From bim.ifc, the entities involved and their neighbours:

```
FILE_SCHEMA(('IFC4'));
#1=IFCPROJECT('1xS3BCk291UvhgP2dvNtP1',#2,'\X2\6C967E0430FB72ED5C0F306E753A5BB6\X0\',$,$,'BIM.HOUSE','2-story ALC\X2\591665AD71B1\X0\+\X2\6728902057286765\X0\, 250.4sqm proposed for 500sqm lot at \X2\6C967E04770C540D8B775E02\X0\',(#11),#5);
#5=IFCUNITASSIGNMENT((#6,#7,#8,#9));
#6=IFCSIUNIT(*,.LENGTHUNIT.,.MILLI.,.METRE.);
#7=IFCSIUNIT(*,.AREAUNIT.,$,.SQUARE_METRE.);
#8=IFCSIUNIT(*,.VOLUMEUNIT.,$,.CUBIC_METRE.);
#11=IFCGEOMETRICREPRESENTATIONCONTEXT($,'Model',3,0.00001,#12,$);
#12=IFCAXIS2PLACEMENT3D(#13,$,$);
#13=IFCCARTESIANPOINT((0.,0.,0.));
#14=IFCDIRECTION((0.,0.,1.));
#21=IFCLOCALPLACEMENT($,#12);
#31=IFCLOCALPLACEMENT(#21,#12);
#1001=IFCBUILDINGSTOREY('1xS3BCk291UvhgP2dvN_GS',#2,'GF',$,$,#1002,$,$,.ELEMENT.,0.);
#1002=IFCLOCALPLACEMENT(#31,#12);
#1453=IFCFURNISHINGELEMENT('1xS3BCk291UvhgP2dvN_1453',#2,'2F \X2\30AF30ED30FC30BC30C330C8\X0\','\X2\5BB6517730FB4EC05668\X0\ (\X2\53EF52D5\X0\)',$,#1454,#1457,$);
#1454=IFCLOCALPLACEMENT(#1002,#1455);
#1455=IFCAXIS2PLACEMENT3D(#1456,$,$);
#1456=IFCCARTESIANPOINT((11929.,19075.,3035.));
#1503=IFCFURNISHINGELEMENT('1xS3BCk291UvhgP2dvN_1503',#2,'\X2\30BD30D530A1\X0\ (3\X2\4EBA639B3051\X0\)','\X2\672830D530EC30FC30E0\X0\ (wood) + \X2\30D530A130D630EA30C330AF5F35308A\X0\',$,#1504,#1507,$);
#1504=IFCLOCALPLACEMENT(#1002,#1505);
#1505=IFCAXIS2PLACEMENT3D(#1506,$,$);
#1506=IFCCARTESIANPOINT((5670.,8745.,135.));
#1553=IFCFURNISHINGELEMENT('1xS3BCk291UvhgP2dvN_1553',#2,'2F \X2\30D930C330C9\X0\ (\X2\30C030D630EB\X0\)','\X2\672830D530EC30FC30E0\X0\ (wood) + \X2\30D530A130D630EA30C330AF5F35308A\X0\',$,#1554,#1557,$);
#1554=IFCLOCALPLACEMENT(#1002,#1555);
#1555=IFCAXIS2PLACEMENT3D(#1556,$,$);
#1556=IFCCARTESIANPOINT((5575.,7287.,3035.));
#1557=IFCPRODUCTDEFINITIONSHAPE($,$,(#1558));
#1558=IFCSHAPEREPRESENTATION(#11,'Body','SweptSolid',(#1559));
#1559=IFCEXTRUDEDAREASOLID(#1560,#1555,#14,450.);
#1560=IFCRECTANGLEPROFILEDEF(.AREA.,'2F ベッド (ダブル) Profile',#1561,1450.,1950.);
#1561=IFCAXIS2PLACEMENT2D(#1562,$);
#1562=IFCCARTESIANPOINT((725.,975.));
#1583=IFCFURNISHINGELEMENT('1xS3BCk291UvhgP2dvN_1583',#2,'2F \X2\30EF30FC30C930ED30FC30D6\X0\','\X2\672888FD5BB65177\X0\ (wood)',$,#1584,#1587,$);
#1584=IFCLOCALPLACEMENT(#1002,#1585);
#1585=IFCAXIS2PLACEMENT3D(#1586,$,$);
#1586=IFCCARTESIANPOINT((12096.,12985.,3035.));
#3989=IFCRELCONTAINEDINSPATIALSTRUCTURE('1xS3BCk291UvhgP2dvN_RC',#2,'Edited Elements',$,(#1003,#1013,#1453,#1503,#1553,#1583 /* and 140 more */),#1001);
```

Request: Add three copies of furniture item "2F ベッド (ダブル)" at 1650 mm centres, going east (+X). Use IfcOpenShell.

```python
import numpy as np
import ifcopenshell
import ifcopenshell.api.geometry
import ifcopenshell.api.root
import ifcopenshell.util.element
import ifcopenshell.util.placement

model = ifcopenshell.open("bim.ifc")


def reuse_history(source, copy):
    """copy_class also copies each property set's owner history, people and application; keep the originals."""
    for rel in copy.IsDefinedBy:
        if rel.is_a("IfcRelDefinesByProperties") and (history := rel.RelatingPropertyDefinition.OwnerHistory):
            rel.RelatingPropertyDefinition.OwnerHistory = source.OwnerHistory
            ifcopenshell.util.element.remove_deep2(model, history)


source = model.by_id(1553)
base = ifcopenshell.util.placement.get_local_placement(source.ObjectPlacement)
step = np.array([1.0, 0.0, 0.0]) * 1650.0

for i in range(1, 4):
    copy = ifcopenshell.api.root.copy_class(model, product=source)
    copy.Representation = ifcopenshell.util.element.copy_deep(
        model, source.Representation, exclude=["IfcGeometricRepresentationContext", "IfcRepresentationMap"]
    )
    reuse_history(source, copy)
    matrix = base.copy()
    matrix[:3, 3] += i * step
    print("added at", matrix[:3, 3].round(3) + 0.0)
    ifcopenshell.api.geometry.edit_object_placement(model, product=copy, matrix=matrix, is_si=False)

model.write("bim_updated.ifc")
```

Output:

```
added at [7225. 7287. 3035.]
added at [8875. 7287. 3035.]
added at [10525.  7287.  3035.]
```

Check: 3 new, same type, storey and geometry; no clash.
